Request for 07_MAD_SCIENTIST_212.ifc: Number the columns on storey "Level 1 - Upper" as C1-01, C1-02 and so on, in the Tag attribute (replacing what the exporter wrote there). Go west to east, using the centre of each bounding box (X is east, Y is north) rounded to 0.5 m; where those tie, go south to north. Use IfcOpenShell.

First a look at what the model holds.

```python
import ifcopenshell
import ifcopenshell.util.element
import ifcopenshell.util.placement

model = ifcopenshell.open("07_MAD_SCIENTIST_212.ifc")
print(model.schema)
storey = next(s for s in model.by_type("IfcBuildingStorey") if s.Name == "Level 1 - Upper")
columns = [e for e in ifcopenshell.util.element.get_decomposition(storey) if e.is_a("IfcColumn")]
for e in sorted(columns, key=lambda e: e.id()):
    origin = ifcopenshell.util.placement.get_local_placement(e.ObjectPlacement)[:3, 3]
    print(e.id(), e.Tag, e.Name, origin.round(2) + 0.0, sep=" | ")
```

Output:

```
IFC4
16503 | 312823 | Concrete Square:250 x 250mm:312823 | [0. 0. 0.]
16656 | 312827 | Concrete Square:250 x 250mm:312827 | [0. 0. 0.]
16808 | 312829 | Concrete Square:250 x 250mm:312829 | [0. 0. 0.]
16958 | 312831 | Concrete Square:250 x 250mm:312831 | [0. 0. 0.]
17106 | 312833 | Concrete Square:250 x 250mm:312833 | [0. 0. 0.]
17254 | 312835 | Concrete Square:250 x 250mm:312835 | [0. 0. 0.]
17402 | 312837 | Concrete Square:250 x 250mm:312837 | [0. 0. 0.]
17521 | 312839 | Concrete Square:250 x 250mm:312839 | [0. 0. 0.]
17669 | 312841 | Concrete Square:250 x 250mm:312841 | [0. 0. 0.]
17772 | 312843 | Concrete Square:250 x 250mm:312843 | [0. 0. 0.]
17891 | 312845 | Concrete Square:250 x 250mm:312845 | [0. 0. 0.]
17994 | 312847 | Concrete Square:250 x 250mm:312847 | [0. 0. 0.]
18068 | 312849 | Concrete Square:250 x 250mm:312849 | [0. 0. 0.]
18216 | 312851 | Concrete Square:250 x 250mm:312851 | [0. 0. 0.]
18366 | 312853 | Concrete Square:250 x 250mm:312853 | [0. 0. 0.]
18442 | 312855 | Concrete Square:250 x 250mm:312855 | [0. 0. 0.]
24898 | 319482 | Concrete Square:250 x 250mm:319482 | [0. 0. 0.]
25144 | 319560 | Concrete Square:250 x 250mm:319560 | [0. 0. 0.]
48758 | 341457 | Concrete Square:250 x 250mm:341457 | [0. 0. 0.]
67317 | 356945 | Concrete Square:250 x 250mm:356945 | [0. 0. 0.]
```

```python
import ifcopenshell
import ifcopenshell.geom
import ifcopenshell.util.element
import ifcopenshell.util.shape

model = ifcopenshell.open("07_MAD_SCIENTIST_212.ifc")
settings = ifcopenshell.geom.settings()
settings.set("use-world-coords", True)


def centre(element):
    shape = ifcopenshell.geom.create_shape(settings, element)
    return ifcopenshell.util.shape.get_bbox_centroid(shape.geometry)


storey = next(s for s in model.by_type("IfcBuildingStorey") if s.Name == "Level 1 - Upper")
columns = [e for e in ifcopenshell.util.element.get_decomposition(storey) if e.is_a("IfcColumn")]

# Insertion points can sit at a corner or the storey origin, so sort by the geometry (in metres).
centres = {e: centre(e) for e in columns}
columns.sort(key=lambda e: (round(centres[e][0] / 0.5), centres[e][1]))

for i, e in enumerate(columns, start=1):
    number = f"C1-{i:02d}"
    e.Tag = number
    print(e.id(), number)

model.write("07_MAD_SCIENTIST_212_updated.ifc")
```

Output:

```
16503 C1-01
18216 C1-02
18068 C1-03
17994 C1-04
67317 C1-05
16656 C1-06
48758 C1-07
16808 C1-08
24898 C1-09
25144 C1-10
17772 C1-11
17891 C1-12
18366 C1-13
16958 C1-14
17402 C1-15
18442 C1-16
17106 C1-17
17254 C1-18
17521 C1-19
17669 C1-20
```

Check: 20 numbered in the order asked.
